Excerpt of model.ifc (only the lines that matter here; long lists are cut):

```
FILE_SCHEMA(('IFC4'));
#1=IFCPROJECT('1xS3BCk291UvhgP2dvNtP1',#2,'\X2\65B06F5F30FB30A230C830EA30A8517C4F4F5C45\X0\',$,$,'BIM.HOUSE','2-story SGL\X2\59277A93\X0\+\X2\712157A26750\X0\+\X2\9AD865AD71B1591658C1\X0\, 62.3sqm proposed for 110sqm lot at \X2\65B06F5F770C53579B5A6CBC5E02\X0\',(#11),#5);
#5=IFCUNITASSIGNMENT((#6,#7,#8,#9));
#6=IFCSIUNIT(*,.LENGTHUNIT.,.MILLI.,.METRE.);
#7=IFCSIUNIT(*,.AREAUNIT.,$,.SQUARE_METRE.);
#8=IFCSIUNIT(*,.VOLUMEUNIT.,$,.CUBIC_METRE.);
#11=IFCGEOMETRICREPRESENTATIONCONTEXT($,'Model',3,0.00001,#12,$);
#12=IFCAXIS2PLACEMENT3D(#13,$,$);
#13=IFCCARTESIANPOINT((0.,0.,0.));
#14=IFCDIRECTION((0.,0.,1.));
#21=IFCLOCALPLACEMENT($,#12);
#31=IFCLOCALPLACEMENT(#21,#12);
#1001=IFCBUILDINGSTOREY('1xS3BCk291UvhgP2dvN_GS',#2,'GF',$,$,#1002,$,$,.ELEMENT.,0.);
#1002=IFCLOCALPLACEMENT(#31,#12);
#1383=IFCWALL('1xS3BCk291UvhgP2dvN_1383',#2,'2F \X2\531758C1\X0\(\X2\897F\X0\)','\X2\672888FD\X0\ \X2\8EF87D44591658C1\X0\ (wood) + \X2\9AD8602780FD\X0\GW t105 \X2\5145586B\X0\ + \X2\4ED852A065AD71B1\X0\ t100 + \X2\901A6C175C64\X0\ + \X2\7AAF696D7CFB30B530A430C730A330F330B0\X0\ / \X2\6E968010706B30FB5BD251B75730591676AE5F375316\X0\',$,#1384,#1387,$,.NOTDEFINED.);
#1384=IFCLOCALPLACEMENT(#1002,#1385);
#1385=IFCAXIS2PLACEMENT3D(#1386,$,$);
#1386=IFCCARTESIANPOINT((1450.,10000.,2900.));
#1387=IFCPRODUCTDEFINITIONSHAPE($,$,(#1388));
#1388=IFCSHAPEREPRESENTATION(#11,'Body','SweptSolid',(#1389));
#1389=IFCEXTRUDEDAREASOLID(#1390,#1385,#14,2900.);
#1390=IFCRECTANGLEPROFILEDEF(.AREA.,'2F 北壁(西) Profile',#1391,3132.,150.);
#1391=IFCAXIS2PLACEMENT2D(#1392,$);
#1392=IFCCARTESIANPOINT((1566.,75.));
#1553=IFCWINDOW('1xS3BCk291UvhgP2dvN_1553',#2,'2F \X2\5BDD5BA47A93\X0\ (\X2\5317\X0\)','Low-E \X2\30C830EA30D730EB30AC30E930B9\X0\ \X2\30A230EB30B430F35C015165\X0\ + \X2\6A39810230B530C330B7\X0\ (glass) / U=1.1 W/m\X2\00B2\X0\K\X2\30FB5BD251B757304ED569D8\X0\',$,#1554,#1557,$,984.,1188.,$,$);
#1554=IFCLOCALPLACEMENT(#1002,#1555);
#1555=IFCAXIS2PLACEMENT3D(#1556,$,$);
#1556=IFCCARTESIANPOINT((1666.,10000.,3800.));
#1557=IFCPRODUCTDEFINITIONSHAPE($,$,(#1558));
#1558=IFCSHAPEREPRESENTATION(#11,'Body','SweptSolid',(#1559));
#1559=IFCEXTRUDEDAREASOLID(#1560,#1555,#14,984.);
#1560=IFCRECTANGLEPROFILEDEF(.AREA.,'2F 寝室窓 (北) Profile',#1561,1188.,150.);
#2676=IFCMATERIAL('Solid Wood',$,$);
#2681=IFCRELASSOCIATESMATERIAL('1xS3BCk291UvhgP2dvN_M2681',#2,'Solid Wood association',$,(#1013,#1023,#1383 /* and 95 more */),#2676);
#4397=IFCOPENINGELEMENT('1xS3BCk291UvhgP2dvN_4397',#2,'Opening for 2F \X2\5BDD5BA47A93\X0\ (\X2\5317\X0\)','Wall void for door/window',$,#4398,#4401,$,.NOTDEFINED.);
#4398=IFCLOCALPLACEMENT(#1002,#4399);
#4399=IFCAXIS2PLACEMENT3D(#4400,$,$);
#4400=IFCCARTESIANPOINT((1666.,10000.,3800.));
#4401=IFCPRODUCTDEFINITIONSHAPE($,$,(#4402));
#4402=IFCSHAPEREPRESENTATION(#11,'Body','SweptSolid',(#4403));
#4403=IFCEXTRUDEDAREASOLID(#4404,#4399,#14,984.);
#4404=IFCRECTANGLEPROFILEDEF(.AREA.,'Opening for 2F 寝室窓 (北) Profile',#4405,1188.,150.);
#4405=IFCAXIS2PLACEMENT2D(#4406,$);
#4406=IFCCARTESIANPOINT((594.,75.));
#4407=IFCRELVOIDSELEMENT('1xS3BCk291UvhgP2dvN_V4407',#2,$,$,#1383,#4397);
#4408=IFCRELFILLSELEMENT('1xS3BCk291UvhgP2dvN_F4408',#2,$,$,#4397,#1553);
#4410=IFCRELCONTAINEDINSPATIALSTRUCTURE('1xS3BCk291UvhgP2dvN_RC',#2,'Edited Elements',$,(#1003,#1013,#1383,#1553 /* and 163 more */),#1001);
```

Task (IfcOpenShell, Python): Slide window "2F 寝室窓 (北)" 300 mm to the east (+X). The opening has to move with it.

```python
import ifcopenshell
import ifcopenshell.api.geometry
import ifcopenshell.util.placement

model = ifcopenshell.open("model.ifc")

window = model.by_guid("1xS3BCk291UvhgP2dvN_1553")
opening = window.FillsVoids[0].RelatingOpeningElement
wall = opening.VoidsElements[0].RelatingBuildingElement

wall_matrix = ifcopenshell.util.placement.get_local_placement(wall.ObjectPlacement)
shift = wall_matrix[:3, 0] * 300.0
before = ifcopenshell.util.placement.get_local_placement(window.ObjectPlacement)[:3, 3].copy()

# The window is not placed relative to its opening, so move both.
for product in (opening, window):
    matrix = ifcopenshell.util.placement.get_local_placement(product.ObjectPlacement)
    matrix[:3, 3] += shift
    ifcopenshell.api.geometry.edit_object_placement(model, product=product, matrix=matrix, is_si=False)

after = ifcopenshell.util.placement.get_local_placement(window.ObjectPlacement)[:3, 3]
print("window moved by", (after - before).round(3) + 0.0)

model.write("model-out.ifc")
```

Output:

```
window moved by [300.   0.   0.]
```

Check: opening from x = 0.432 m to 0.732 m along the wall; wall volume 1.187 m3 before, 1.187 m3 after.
